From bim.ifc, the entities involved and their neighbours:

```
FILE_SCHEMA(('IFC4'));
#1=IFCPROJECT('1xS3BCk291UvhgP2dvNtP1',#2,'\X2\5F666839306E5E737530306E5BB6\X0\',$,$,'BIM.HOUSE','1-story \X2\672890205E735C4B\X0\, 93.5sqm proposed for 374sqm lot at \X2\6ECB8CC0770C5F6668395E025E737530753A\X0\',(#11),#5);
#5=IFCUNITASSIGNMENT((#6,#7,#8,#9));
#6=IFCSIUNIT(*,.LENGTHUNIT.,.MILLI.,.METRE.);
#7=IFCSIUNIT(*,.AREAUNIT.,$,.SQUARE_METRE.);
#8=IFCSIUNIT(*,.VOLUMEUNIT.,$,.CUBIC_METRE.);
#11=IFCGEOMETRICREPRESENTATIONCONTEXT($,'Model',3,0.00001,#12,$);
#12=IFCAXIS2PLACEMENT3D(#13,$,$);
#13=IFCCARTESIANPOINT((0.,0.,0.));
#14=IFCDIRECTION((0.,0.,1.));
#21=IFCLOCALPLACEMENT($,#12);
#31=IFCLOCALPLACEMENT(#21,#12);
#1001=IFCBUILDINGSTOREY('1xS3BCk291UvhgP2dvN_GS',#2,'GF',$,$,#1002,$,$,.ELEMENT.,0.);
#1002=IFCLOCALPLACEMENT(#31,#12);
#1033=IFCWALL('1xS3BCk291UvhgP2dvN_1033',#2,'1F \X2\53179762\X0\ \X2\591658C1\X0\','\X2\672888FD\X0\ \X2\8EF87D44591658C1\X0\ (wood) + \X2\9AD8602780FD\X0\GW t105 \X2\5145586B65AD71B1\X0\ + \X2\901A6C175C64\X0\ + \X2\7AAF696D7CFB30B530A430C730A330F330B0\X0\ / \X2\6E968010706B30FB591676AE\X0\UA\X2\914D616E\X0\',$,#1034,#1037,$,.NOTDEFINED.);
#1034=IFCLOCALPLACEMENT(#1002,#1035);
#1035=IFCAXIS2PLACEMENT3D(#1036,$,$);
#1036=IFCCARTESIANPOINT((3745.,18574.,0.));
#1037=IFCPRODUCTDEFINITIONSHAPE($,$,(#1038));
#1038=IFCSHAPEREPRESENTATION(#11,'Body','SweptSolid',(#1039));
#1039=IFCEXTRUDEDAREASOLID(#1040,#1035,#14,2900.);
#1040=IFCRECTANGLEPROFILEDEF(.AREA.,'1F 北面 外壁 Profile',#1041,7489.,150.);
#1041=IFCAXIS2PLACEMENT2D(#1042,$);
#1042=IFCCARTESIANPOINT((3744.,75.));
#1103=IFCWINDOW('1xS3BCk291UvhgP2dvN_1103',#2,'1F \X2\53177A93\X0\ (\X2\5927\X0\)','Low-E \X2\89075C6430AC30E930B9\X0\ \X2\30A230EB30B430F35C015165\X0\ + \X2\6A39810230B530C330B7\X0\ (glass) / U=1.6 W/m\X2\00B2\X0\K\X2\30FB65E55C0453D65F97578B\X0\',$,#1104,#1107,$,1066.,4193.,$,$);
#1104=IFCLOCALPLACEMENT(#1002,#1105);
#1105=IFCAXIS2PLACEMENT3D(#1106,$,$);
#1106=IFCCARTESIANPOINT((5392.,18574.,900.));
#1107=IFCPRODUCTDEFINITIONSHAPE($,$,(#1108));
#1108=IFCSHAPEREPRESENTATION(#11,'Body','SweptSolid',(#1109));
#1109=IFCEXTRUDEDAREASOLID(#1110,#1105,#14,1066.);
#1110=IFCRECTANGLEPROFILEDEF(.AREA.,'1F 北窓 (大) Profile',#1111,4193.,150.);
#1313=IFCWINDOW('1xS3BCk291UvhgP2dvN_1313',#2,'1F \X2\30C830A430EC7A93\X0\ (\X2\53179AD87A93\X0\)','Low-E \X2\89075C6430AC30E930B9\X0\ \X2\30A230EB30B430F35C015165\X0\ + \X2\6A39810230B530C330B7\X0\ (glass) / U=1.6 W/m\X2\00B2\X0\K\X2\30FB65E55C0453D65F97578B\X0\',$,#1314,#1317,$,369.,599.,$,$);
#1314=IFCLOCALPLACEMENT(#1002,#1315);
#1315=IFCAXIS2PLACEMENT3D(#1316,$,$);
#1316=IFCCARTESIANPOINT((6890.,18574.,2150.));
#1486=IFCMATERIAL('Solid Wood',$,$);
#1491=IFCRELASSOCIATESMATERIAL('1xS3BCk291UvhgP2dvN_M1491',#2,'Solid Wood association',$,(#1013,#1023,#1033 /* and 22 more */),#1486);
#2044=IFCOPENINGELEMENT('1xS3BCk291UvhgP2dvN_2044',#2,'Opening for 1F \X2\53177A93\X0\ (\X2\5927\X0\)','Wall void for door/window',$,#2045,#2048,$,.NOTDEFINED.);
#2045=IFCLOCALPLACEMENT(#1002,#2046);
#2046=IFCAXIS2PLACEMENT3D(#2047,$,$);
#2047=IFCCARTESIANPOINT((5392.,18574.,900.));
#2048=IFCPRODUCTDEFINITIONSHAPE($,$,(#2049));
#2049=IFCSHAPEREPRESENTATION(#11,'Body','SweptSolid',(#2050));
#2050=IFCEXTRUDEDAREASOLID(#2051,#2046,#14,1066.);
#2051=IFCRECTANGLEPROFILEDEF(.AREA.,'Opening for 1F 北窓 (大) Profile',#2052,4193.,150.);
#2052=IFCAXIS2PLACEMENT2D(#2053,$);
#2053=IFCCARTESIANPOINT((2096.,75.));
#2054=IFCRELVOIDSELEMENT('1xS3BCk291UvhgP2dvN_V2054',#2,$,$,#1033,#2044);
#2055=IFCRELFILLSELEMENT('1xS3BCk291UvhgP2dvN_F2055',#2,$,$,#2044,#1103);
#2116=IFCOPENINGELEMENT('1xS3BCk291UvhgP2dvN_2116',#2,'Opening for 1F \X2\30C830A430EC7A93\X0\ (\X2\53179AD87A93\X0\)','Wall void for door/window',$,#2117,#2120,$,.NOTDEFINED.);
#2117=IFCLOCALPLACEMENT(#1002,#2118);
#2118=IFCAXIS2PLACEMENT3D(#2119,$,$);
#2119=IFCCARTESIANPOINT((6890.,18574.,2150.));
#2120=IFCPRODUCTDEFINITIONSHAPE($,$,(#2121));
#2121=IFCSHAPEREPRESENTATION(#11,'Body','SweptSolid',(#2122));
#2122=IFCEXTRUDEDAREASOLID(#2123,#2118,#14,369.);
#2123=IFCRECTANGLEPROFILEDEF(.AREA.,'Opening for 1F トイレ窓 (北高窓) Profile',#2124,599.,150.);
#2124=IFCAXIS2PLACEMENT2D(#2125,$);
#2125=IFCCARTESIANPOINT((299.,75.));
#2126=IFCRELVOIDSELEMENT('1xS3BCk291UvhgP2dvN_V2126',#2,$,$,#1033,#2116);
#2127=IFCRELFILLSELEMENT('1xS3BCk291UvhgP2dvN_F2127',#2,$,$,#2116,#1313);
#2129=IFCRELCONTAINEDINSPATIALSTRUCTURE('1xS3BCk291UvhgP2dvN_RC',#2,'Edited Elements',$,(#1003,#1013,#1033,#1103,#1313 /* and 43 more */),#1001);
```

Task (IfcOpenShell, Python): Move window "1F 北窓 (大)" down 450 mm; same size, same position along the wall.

```python
import numpy as np
import ifcopenshell
import ifcopenshell.api.geometry
import ifcopenshell.util.placement
import ifcopenshell.util.unit

model = ifcopenshell.open("bim.ifc")
unit_scale = ifcopenshell.util.unit.calculate_unit_scale(model)

window = model.by_guid("1xS3BCk291UvhgP2dvN_1103")
opening = window.FillsVoids[0].RelatingOpeningElement
dz = -0.45 / unit_scale

shift = np.array([0.0, 0.0, dz])
# The window is not placed relative to its opening, so move both.
for product in (opening, window):
    matrix = ifcopenshell.util.placement.get_local_placement(product.ObjectPlacement)
    matrix[:3, 3] += shift
    ifcopenshell.api.geometry.edit_object_placement(model, product=product, matrix=matrix, is_si=False)

print(f"moved by {dz * unit_scale:+.3f} m")

model.write("bim_v2.ifc")
```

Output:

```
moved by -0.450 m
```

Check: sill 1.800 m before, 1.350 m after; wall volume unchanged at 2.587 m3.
